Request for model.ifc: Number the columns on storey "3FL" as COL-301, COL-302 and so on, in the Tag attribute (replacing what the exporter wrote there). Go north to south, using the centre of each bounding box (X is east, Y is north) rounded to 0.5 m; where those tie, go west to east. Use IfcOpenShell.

First a look at what the model holds.

```python
import ifcopenshell
import ifcopenshell.util.element
import ifcopenshell.util.placement

model = ifcopenshell.open("model.ifc")
print(model.schema)
storey = next(s for s in model.by_type("IfcBuildingStorey") if s.Name == "3FL")
columns = [e for e in ifcopenshell.util.element.get_decomposition(storey) if e.is_a("IfcColumn")]
for e in sorted(columns, key=lambda e: e.id()):
    origin = ifcopenshell.util.placement.get_local_placement(e.ObjectPlacement)[:3, 3]
    print(e.id(), e.Tag, e.Name, origin.round(2) + 0.0, sep=" | ")
```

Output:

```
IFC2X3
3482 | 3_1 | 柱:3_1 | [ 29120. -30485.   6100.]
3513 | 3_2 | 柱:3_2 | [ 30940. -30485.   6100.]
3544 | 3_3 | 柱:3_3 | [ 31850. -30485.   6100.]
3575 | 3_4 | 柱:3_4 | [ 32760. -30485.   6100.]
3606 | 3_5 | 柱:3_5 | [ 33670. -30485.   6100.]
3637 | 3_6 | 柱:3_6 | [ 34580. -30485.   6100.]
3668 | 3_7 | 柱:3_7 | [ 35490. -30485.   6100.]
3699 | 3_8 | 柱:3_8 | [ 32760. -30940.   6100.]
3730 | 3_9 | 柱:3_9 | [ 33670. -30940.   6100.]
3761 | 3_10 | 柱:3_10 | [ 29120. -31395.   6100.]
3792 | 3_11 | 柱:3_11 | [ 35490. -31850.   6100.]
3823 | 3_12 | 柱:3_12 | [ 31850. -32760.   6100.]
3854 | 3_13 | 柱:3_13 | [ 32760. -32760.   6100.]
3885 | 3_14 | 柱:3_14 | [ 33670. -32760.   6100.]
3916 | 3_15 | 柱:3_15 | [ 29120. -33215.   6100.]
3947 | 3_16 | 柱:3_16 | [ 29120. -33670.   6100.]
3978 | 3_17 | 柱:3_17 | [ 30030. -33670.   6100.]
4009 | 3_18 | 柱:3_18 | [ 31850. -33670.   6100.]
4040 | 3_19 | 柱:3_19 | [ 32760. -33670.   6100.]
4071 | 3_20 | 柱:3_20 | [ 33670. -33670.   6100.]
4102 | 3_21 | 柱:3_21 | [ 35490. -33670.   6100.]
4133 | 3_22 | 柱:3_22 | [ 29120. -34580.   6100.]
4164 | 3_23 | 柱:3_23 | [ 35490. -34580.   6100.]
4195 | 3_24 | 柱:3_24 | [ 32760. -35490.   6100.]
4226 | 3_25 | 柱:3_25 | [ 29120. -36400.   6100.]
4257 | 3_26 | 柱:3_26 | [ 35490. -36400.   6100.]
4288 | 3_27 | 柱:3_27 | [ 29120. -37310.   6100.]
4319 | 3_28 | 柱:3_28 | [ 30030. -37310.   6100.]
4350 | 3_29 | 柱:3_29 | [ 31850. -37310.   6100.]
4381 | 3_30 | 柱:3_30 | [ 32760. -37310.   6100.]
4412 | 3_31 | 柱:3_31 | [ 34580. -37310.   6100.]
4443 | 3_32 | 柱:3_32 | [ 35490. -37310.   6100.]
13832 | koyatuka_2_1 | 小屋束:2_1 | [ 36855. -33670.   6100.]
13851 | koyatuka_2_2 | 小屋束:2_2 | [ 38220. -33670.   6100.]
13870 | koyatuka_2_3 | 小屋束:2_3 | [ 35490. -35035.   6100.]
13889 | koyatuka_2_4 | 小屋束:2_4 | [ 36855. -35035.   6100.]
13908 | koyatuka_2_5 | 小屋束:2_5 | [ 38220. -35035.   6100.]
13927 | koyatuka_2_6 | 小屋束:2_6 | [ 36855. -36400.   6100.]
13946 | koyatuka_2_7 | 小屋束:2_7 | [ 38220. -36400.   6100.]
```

```python
import ifcopenshell
import ifcopenshell.geom
import ifcopenshell.util.element
import ifcopenshell.util.shape

model = ifcopenshell.open("model.ifc")
settings = ifcopenshell.geom.settings()
settings.set("use-world-coords", True)


def centre(element):
    shape = ifcopenshell.geom.create_shape(settings, element)
    return ifcopenshell.util.shape.get_bbox_centroid(shape.geometry)


storey = next(s for s in model.by_type("IfcBuildingStorey") if s.Name == "3FL")
columns = [e for e in ifcopenshell.util.element.get_decomposition(storey) if e.is_a("IfcColumn")]

# Insertion points can sit at a corner or the storey origin, so sort by the geometry (in metres).
centres = {e: centre(e) for e in columns}
columns.sort(key=lambda e: (-round(centres[e][1] / 0.5), centres[e][0]))

for i, e in enumerate(columns, start=1):
    number = f"COL-3{i:02d}"
    e.Tag = number
    print(e.id(), number)

model.write("model_rev.ifc")
```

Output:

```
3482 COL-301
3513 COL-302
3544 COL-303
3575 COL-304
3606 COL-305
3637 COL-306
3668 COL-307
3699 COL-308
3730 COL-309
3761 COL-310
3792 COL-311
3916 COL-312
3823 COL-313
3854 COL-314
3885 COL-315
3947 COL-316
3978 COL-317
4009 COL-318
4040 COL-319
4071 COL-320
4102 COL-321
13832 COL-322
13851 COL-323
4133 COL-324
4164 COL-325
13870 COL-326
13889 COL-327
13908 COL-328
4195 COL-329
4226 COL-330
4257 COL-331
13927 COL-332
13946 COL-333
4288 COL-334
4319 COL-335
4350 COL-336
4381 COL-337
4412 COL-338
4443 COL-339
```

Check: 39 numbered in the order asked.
